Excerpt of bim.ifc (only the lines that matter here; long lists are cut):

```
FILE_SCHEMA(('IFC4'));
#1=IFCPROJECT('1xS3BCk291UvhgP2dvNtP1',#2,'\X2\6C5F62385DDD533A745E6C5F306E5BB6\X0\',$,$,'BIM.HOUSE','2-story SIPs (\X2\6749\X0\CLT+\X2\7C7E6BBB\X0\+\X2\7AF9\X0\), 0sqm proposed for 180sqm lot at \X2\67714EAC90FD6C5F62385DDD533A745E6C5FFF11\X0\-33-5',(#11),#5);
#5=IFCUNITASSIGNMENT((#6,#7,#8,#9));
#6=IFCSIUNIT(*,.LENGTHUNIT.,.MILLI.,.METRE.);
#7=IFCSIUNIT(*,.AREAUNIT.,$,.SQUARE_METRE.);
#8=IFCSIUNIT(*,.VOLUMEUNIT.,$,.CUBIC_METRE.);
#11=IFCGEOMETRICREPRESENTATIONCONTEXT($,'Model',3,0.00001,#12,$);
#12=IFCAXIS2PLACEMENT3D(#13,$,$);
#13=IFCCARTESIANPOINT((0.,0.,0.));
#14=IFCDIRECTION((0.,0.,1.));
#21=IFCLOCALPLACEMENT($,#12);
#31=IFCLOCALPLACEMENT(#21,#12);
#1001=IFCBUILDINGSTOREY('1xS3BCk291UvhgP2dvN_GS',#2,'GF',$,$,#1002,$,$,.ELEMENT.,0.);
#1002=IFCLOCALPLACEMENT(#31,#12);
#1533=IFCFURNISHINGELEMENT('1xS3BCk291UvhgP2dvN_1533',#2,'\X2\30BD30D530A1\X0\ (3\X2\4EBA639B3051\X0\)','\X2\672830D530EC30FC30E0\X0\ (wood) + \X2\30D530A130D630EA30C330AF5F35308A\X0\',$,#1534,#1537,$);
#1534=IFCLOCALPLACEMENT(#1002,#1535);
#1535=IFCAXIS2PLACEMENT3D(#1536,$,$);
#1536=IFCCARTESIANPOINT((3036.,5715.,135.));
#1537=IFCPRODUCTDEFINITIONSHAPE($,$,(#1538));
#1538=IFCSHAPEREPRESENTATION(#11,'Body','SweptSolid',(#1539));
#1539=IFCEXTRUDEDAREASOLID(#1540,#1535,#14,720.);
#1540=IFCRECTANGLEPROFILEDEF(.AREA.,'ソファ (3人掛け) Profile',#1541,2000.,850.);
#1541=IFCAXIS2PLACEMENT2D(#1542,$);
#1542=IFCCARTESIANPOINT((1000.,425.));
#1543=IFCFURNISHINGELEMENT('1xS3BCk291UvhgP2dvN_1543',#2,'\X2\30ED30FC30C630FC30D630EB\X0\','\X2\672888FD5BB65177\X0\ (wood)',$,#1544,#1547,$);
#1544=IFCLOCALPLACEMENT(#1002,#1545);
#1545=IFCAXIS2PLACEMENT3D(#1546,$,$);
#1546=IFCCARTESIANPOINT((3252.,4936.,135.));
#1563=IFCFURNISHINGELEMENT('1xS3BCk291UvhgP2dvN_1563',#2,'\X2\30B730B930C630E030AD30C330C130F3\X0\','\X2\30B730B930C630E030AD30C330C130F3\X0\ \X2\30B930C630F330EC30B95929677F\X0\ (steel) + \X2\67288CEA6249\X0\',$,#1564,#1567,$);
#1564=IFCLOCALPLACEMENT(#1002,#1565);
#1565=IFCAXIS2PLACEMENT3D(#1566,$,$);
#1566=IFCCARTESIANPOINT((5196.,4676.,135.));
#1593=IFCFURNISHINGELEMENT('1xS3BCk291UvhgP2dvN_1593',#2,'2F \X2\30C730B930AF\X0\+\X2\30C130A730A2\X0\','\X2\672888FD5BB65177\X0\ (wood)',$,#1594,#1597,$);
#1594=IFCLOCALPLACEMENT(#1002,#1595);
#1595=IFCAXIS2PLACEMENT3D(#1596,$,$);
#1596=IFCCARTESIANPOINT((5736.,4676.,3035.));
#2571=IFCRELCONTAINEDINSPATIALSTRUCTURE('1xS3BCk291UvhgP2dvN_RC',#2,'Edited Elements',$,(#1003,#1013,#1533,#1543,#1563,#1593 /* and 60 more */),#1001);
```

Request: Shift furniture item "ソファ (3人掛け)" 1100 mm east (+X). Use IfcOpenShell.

```python
import ifcopenshell
import ifcopenshell.api.geometry
import ifcopenshell.util.placement
import ifcopenshell.util.unit

model = ifcopenshell.open("bim.ifc")
unit_scale = ifcopenshell.util.unit.calculate_unit_scale(model)

item = model.by_guid("1xS3BCk291UvhgP2dvN_1533")
matrix = ifcopenshell.util.placement.get_local_placement(item.ObjectPlacement)
matrix[0, 3] += 1.1 / unit_scale
ifcopenshell.api.geometry.edit_object_placement(model, product=item, matrix=matrix, is_si=False)

print(ifcopenshell.util.placement.get_local_placement(item.ObjectPlacement).round(3) + 0.0)

model.write("bim_v2.ifc")
```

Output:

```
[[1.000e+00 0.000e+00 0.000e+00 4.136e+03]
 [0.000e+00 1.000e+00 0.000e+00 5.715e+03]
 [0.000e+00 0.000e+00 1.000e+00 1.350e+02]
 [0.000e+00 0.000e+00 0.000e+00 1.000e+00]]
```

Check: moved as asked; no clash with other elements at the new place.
